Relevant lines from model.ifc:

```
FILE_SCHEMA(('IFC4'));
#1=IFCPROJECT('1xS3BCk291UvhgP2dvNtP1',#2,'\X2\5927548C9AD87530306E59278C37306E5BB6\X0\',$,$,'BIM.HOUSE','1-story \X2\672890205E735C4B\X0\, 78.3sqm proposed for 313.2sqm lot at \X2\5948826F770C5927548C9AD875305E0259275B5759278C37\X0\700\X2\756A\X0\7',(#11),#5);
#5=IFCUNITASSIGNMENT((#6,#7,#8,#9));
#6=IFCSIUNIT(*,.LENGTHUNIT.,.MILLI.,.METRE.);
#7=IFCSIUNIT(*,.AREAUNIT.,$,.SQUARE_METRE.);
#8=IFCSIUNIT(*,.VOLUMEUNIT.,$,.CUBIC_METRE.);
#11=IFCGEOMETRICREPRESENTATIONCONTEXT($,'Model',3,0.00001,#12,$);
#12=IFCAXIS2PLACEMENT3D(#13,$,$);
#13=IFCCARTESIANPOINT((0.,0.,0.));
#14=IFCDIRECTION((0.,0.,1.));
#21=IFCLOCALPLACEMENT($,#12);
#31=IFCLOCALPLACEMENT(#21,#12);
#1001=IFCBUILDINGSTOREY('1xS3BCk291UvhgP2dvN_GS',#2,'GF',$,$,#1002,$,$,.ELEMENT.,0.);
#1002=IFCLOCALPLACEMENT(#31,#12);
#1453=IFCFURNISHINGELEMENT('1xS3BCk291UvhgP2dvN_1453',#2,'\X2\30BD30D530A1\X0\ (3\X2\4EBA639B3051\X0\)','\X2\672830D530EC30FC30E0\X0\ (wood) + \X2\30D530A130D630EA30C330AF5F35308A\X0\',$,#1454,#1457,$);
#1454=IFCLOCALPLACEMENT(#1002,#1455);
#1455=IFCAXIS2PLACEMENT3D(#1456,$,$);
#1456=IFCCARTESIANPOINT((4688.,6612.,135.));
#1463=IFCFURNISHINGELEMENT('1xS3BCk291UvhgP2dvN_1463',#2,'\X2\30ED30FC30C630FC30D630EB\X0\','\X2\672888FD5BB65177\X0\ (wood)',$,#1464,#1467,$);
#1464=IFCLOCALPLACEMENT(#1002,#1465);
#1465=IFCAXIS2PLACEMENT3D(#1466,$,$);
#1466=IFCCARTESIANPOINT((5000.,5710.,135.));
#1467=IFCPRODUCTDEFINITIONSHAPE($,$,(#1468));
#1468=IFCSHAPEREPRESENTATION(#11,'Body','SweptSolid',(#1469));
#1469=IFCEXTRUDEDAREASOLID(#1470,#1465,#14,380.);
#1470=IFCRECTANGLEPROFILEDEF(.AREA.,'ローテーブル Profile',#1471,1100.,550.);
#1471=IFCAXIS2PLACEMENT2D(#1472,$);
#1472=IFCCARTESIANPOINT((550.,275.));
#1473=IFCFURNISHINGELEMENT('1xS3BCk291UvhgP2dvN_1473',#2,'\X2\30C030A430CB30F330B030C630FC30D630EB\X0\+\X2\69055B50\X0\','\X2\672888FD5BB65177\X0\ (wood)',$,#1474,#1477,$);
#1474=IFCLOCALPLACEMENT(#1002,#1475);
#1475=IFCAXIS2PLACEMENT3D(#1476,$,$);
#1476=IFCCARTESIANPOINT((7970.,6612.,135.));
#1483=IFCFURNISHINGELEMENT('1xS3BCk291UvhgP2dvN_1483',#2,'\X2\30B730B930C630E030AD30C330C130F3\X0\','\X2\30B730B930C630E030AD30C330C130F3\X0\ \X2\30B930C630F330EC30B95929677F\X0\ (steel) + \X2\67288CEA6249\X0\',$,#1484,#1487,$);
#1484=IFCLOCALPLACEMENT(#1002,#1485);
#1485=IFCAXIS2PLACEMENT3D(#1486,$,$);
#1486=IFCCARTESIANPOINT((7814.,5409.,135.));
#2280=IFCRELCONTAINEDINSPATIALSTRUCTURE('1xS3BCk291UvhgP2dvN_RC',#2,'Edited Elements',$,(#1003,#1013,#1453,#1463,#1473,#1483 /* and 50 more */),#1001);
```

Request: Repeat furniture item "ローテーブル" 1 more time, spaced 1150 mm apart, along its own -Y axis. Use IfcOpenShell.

```python
import ifcopenshell
import ifcopenshell.api.geometry
import ifcopenshell.api.root
import ifcopenshell.util.element
import ifcopenshell.util.placement
import ifcopenshell.util.unit

model = ifcopenshell.open("model.ifc")
unit_scale = ifcopenshell.util.unit.calculate_unit_scale(model)


def reuse_history(source, copy):
    """copy_class also copies each property set's owner history, people and application; keep the originals."""
    for rel in copy.IsDefinedBy:
        if rel.is_a("IfcRelDefinesByProperties") and (history := rel.RelatingPropertyDefinition.OwnerHistory):
            rel.RelatingPropertyDefinition.OwnerHistory = source.OwnerHistory
            ifcopenshell.util.element.remove_deep2(model, history)


source = model.by_guid("1xS3BCk291UvhgP2dvN_1463")
base = ifcopenshell.util.placement.get_local_placement(source.ObjectPlacement)
step = -base[:3, 1] * 1.15 / unit_scale

for i in range(1, 2):
    copy = ifcopenshell.api.root.copy_class(model, product=source)
    copy.Representation = ifcopenshell.util.element.copy_deep(
        model, source.Representation, exclude=["IfcGeometricRepresentationContext", "IfcRepresentationMap"]
    )
    reuse_history(source, copy)
    matrix = base.copy()
    matrix[:3, 3] += i * step
    print("added at", matrix[:3, 3].round(3) + 0.0)
    ifcopenshell.api.geometry.edit_object_placement(model, product=copy, matrix=matrix, is_si=False)

model.write("model_edited.ifc")
```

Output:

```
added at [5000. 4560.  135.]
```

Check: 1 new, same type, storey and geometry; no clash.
